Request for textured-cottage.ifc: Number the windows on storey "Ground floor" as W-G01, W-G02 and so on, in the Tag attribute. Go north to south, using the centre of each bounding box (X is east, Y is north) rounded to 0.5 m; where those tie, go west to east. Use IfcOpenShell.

First a look at what the model holds.

```python
import ifcopenshell
import ifcopenshell.util.element
import ifcopenshell.util.placement

model = ifcopenshell.open("textured-cottage.ifc")
print(model.schema)
storey = next(s for s in model.by_type("IfcBuildingStorey") if s.Name == "Ground floor")
windows = [e for e in ifcopenshell.util.element.get_decomposition(storey) if e.is_a("IfcWindow")]
for e in sorted(windows, key=lambda e: e.id()):
    origin = ifcopenshell.util.placement.get_local_placement(e.ObjectPlacement)[:3, 3]
    print(e.id(), e.Tag, e.Name, origin.round(2) + 0.0, sep=" | ")
```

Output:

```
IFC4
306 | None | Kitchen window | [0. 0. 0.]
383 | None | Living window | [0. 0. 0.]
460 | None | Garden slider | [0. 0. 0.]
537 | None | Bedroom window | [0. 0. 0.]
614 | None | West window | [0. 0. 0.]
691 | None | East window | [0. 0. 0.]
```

```python
import ifcopenshell
import ifcopenshell.geom
import ifcopenshell.util.element
import ifcopenshell.util.shape

model = ifcopenshell.open("textured-cottage.ifc")
settings = ifcopenshell.geom.settings()
settings.set("use-world-coords", True)


def centre(element):
    shape = ifcopenshell.geom.create_shape(settings, element)
    return ifcopenshell.util.shape.get_bbox_centroid(shape.geometry)


storey = next(s for s in model.by_type("IfcBuildingStorey") if s.Name == "Ground floor")
windows = [e for e in ifcopenshell.util.element.get_decomposition(storey) if e.is_a("IfcWindow")]

# Insertion points can sit at a corner or the storey origin, so sort by the geometry (in metres).
centres = {e: centre(e) for e in windows}
windows.sort(key=lambda e: (-round(centres[e][1] / 0.5), centres[e][0]))

for i, e in enumerate(windows, start=1):
    number = f"W-G{i:02d}"
    e.Tag = number
    print(e.id(), number)

model.write("textured-cottage_rev.ifc")
```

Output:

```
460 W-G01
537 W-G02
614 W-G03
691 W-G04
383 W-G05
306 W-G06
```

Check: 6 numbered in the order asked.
